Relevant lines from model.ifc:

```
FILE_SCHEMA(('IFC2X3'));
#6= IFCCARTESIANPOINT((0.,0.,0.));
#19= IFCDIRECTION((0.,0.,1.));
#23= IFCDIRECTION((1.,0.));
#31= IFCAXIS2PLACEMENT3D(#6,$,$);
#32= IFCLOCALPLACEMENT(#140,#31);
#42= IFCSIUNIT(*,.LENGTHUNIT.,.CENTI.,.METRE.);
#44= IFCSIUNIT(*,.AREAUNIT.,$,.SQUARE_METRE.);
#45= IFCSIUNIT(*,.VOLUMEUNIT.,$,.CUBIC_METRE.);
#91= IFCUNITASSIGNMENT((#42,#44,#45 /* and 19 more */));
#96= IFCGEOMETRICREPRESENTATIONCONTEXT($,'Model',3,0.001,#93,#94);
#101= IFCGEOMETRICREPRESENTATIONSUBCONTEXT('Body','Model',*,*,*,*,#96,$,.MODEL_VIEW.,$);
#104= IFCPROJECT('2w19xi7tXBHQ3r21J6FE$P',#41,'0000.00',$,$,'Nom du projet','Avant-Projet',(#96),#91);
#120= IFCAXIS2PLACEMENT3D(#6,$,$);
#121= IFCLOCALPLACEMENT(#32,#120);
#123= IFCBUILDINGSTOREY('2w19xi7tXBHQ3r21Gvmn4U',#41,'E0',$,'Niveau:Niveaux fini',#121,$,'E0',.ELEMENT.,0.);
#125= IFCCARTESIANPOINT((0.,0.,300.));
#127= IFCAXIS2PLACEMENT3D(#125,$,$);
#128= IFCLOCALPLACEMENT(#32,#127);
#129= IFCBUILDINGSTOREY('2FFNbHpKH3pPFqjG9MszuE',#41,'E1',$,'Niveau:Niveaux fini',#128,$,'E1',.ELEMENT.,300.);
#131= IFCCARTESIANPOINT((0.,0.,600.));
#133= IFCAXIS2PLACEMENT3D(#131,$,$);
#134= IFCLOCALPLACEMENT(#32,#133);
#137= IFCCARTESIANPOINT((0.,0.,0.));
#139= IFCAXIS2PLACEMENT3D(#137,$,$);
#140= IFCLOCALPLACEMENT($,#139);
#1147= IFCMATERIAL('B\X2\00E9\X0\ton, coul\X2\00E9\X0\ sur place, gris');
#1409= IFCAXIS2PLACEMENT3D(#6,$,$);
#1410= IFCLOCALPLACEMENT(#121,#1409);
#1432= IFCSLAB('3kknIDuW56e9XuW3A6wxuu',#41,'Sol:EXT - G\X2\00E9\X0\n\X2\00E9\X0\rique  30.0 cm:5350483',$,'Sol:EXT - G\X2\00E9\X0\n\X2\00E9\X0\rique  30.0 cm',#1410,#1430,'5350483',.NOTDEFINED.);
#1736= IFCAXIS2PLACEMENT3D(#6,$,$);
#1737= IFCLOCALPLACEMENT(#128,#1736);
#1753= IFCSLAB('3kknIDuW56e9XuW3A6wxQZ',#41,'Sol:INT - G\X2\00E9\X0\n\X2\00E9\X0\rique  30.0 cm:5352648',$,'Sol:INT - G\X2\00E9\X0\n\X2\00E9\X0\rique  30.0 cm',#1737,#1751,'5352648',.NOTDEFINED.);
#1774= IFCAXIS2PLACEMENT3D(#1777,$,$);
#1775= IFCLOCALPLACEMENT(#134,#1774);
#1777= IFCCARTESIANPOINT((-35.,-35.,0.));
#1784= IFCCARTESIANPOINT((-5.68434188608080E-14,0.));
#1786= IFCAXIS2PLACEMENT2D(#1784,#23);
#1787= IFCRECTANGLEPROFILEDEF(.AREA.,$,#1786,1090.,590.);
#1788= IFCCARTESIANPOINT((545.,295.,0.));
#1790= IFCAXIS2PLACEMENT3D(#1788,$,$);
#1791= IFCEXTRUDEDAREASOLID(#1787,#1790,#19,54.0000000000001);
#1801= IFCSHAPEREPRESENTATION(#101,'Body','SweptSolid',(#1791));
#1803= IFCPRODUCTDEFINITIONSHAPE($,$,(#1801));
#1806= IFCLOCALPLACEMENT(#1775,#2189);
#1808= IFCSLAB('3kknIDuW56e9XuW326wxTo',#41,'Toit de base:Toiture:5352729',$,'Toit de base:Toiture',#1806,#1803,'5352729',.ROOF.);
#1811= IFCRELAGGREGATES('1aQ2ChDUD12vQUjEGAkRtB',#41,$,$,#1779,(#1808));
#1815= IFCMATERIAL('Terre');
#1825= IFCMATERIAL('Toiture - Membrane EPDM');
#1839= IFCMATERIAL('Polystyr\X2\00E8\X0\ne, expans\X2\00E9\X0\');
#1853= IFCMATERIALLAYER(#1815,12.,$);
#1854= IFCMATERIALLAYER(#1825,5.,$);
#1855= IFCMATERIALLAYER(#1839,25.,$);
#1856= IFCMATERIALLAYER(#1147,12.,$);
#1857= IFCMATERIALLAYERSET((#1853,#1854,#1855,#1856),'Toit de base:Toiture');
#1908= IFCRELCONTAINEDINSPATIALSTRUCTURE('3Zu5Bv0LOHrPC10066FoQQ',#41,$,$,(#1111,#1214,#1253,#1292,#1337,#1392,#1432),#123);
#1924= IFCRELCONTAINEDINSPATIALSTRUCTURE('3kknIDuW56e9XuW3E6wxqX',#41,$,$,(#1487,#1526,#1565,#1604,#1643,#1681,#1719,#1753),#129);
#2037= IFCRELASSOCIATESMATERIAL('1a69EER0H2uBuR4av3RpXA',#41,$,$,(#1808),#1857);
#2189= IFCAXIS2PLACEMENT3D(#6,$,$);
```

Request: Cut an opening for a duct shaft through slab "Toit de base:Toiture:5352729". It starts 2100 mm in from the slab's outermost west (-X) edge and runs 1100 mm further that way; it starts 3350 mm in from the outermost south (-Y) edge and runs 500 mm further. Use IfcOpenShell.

```python
import numpy as np
import ifcopenshell
import ifcopenshell.api.feature
import ifcopenshell.api.geometry
import ifcopenshell.api.root
import ifcopenshell.geom
import ifcopenshell.util.placement
import ifcopenshell.util.representation
import ifcopenshell.util.shape
import ifcopenshell.util.unit

model = ifcopenshell.open("model.ifc")
unit_scale = ifcopenshell.util.unit.calculate_unit_scale(model)
settings = ifcopenshell.geom.settings()


def volume(element):
    """Net volume in cubic metres, openings subtracted."""
    shape = ifcopenshell.geom.create_shape(settings, element)
    return ifcopenshell.util.shape.get_volume(shape.geometry)


slab = model.by_id(1808)
before = volume(slab)

# Extent in the slab's own axes, in metres. The edges named are its -X and -Y sides.
slab_shape = ifcopenshell.geom.create_shape(settings, slab)
vertices = ifcopenshell.util.shape.get_vertices(slab_shape.geometry)
x_min, y_min, bottom = vertices.min(axis=0)
top = vertices[:, 2].max()

opening = ifcopenshell.api.root.create_entity(model, ifc_class="IfcOpeningElement", name="Duct shaft opening")
context = ifcopenshell.util.representation.get_context(model, "Model", "Body", "MODEL_VIEW")
width, depth = 1.1, 0.5
outline = [(0.0, 0.0), (width, 0.0), (width, depth), (0.0, depth), (0.0, 0.0)]
# Overshoot both faces by 50 mm so the cut is clean.
shape = ifcopenshell.api.geometry.add_slab_representation(
    model, context=context, depth=top - bottom + 0.1, polyline=outline
)
ifcopenshell.api.geometry.assign_representation(model, product=opening, representation=shape)

matrix = ifcopenshell.util.placement.get_local_placement(slab.ObjectPlacement)
matrix[:, 3] = matrix @ np.append(np.array([x_min + 2.1, y_min + 3.35, bottom - 0.05]) / unit_scale, 1.0)
ifcopenshell.api.geometry.edit_object_placement(model, product=opening, matrix=matrix, is_si=False)
ifcopenshell.api.feature.add_feature(model, feature=opening, element=slab)

after = volume(slab)

print(f"slab volume {before:.3f} -> {after:.3f} m3")

model.write("model_rev.ifc")
```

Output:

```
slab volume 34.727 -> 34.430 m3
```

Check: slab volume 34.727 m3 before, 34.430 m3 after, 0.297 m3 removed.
